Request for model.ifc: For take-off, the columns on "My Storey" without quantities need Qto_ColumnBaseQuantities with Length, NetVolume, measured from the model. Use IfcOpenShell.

First a look at what the model holds.

```python
import ifcopenshell
import ifcopenshell.util.element
import ifcopenshell.util.unit

model = ifcopenshell.open("model.ifc")
print(model.schema)
for unit_type in ("LENGTHUNIT", "AREAUNIT", "VOLUMEUNIT"):
    print(unit_type, ifcopenshell.util.unit.calculate_unit_scale(model, unit_type))
storey = next(s for s in model.by_type("IfcBuildingStorey") if s.Name == "My Storey")
columns = [e for e in ifcopenshell.util.element.get_decomposition(storey) if e.is_a("IfcColumn")]
for e in sorted(columns, key=lambda e: e.id()):
    print(e.id(), e.is_a(), e.Name, list(ifcopenshell.util.element.get_psets(e, qtos_only=True)), sep=" | ")
```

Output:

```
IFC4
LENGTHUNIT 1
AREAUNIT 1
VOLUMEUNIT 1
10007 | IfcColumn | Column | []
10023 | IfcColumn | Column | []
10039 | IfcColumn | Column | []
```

```python
import ifcopenshell
import ifcopenshell.api.pset
import ifcopenshell.geom
import ifcopenshell.util.element
import ifcopenshell.util.shape
import ifcopenshell.util.unit

model = ifcopenshell.open("model.ifc")
unit_scale = ifcopenshell.util.unit.calculate_unit_scale(model)
volume_scale = ifcopenshell.util.unit.calculate_unit_scale(model, "VOLUMEUNIT")
settings = ifcopenshell.geom.settings()

storey = next(s for s in model.by_type("IfcBuildingStorey") if s.Name == "My Storey")
columns = [e for e in ifcopenshell.util.element.get_decomposition(storey) if e.is_a("IfcColumn")]

for e in sorted(columns, key=lambda e: e.id()):
    if ifcopenshell.util.element.get_psets(e, qtos_only=True, should_inherit=False):
        continue
    # Geometry comes back in metres, in the element's own axes.
    shape = ifcopenshell.geom.create_shape(settings, e)
    values = {
        "Length": ifcopenshell.util.shape.get_z(shape.geometry) / unit_scale,
        "NetVolume": ifcopenshell.util.shape.get_volume(shape.geometry) / volume_scale,
    }
    qto = ifcopenshell.api.pset.add_qto(model, product=e, name="Qto_ColumnBaseQuantities")
    ifcopenshell.api.pset.edit_qto(model, qto=qto, properties=values)
    print(e.id(), {k: round(v, 3) for k, v in values.items()})

model.write("model_edited.ifc")
```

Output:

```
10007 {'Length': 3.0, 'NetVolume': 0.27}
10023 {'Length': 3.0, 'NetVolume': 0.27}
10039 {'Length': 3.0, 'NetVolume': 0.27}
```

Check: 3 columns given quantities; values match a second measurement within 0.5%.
